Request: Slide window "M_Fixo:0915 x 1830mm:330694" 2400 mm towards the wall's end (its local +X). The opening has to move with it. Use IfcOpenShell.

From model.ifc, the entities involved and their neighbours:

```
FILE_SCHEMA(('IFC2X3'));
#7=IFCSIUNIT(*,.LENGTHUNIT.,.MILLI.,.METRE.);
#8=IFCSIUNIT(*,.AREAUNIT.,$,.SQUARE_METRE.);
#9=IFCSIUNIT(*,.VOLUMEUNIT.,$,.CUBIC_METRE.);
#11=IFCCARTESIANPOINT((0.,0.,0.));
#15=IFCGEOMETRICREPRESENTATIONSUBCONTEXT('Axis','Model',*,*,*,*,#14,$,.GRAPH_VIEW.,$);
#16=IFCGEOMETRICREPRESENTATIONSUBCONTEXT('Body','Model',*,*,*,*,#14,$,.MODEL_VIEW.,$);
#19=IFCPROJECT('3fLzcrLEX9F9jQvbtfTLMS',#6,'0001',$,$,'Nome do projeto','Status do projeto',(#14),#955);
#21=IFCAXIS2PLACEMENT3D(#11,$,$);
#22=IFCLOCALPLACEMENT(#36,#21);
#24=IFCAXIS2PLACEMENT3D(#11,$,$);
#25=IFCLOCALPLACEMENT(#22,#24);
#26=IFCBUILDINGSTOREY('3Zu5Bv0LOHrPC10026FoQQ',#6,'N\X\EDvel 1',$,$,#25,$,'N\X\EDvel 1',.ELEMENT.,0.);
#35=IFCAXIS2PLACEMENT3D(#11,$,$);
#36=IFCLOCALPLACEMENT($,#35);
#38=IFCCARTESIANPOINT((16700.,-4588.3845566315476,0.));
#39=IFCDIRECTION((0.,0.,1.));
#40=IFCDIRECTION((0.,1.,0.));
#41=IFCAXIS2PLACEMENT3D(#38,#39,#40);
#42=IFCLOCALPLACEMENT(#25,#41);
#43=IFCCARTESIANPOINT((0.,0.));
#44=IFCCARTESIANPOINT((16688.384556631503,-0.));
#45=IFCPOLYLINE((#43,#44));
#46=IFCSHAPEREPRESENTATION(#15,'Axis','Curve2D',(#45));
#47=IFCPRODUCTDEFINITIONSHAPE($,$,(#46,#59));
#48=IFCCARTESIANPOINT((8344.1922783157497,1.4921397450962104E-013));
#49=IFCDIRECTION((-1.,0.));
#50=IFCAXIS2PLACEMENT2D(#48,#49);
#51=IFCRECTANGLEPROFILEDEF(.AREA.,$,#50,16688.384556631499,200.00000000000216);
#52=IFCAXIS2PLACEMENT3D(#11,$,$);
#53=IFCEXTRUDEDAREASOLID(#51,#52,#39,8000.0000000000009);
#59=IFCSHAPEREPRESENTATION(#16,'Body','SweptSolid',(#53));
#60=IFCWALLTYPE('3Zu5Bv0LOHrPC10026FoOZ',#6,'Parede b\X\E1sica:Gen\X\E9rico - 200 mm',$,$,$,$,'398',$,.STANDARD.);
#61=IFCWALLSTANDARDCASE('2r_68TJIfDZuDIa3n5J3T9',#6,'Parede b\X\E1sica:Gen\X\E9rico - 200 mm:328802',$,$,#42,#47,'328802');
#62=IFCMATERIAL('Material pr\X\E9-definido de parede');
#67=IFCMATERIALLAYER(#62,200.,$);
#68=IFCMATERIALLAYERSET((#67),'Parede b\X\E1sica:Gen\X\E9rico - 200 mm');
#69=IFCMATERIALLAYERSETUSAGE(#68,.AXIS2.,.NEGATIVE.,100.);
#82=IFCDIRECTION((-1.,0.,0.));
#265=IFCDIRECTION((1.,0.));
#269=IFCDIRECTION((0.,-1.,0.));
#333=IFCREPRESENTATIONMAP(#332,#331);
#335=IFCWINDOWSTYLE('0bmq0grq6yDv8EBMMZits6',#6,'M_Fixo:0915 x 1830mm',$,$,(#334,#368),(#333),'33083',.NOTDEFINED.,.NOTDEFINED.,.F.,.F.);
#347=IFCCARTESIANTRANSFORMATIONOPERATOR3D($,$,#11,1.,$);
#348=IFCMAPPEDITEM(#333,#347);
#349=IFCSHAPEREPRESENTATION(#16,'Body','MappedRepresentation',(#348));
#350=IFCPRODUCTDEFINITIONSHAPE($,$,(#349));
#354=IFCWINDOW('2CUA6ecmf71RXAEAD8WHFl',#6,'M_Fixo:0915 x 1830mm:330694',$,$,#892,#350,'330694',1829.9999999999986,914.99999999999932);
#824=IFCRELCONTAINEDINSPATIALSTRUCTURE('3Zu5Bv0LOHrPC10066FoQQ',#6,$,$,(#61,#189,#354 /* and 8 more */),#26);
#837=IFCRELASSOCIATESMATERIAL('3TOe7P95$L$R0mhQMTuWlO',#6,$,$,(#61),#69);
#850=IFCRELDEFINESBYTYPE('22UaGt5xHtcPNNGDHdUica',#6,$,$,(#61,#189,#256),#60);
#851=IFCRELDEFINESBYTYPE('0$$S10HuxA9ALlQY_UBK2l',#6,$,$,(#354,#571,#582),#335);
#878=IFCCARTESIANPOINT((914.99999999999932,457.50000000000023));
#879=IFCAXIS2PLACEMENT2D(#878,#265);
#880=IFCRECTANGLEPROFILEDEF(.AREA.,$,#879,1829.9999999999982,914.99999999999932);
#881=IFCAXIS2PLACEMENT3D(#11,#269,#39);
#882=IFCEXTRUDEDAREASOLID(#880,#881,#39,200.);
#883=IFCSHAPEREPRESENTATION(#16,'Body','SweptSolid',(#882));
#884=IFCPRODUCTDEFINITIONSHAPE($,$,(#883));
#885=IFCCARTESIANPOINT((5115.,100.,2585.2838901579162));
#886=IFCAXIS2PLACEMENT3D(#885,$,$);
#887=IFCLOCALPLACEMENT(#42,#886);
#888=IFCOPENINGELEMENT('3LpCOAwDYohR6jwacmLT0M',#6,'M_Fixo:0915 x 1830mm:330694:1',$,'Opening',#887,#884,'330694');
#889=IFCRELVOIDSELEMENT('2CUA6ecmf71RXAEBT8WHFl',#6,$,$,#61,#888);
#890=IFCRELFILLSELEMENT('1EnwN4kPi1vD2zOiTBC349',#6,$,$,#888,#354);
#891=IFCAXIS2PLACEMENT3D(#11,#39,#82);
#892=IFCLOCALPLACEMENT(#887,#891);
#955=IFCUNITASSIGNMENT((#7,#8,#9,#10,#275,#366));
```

```python
import ifcopenshell
import ifcopenshell.api.geometry
import ifcopenshell.util.placement

model = ifcopenshell.open("model.ifc")

window = model.by_id(354)
opening = window.FillsVoids[0].RelatingOpeningElement
wall = opening.VoidsElements[0].RelatingBuildingElement

wall_matrix = ifcopenshell.util.placement.get_local_placement(wall.ObjectPlacement)
shift = wall_matrix[:3, 0] * 2400.0
before = ifcopenshell.util.placement.get_local_placement(window.ObjectPlacement)[:3, 3].copy()

# The window is placed relative to its opening, so it follows when the opening moves.
matrix = ifcopenshell.util.placement.get_local_placement(opening.ObjectPlacement)
matrix[:3, 3] += shift
ifcopenshell.api.geometry.edit_object_placement(
    model, product=opening, matrix=matrix, is_si=False, should_transform_children=True
)

after = ifcopenshell.util.placement.get_local_placement(window.ObjectPlacement)[:3, 3]
print("window moved by", (after - before).round(3) + 0.0)

model.write("model_rev.ifc")
```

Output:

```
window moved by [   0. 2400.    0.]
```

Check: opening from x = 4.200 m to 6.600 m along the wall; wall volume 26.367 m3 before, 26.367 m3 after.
